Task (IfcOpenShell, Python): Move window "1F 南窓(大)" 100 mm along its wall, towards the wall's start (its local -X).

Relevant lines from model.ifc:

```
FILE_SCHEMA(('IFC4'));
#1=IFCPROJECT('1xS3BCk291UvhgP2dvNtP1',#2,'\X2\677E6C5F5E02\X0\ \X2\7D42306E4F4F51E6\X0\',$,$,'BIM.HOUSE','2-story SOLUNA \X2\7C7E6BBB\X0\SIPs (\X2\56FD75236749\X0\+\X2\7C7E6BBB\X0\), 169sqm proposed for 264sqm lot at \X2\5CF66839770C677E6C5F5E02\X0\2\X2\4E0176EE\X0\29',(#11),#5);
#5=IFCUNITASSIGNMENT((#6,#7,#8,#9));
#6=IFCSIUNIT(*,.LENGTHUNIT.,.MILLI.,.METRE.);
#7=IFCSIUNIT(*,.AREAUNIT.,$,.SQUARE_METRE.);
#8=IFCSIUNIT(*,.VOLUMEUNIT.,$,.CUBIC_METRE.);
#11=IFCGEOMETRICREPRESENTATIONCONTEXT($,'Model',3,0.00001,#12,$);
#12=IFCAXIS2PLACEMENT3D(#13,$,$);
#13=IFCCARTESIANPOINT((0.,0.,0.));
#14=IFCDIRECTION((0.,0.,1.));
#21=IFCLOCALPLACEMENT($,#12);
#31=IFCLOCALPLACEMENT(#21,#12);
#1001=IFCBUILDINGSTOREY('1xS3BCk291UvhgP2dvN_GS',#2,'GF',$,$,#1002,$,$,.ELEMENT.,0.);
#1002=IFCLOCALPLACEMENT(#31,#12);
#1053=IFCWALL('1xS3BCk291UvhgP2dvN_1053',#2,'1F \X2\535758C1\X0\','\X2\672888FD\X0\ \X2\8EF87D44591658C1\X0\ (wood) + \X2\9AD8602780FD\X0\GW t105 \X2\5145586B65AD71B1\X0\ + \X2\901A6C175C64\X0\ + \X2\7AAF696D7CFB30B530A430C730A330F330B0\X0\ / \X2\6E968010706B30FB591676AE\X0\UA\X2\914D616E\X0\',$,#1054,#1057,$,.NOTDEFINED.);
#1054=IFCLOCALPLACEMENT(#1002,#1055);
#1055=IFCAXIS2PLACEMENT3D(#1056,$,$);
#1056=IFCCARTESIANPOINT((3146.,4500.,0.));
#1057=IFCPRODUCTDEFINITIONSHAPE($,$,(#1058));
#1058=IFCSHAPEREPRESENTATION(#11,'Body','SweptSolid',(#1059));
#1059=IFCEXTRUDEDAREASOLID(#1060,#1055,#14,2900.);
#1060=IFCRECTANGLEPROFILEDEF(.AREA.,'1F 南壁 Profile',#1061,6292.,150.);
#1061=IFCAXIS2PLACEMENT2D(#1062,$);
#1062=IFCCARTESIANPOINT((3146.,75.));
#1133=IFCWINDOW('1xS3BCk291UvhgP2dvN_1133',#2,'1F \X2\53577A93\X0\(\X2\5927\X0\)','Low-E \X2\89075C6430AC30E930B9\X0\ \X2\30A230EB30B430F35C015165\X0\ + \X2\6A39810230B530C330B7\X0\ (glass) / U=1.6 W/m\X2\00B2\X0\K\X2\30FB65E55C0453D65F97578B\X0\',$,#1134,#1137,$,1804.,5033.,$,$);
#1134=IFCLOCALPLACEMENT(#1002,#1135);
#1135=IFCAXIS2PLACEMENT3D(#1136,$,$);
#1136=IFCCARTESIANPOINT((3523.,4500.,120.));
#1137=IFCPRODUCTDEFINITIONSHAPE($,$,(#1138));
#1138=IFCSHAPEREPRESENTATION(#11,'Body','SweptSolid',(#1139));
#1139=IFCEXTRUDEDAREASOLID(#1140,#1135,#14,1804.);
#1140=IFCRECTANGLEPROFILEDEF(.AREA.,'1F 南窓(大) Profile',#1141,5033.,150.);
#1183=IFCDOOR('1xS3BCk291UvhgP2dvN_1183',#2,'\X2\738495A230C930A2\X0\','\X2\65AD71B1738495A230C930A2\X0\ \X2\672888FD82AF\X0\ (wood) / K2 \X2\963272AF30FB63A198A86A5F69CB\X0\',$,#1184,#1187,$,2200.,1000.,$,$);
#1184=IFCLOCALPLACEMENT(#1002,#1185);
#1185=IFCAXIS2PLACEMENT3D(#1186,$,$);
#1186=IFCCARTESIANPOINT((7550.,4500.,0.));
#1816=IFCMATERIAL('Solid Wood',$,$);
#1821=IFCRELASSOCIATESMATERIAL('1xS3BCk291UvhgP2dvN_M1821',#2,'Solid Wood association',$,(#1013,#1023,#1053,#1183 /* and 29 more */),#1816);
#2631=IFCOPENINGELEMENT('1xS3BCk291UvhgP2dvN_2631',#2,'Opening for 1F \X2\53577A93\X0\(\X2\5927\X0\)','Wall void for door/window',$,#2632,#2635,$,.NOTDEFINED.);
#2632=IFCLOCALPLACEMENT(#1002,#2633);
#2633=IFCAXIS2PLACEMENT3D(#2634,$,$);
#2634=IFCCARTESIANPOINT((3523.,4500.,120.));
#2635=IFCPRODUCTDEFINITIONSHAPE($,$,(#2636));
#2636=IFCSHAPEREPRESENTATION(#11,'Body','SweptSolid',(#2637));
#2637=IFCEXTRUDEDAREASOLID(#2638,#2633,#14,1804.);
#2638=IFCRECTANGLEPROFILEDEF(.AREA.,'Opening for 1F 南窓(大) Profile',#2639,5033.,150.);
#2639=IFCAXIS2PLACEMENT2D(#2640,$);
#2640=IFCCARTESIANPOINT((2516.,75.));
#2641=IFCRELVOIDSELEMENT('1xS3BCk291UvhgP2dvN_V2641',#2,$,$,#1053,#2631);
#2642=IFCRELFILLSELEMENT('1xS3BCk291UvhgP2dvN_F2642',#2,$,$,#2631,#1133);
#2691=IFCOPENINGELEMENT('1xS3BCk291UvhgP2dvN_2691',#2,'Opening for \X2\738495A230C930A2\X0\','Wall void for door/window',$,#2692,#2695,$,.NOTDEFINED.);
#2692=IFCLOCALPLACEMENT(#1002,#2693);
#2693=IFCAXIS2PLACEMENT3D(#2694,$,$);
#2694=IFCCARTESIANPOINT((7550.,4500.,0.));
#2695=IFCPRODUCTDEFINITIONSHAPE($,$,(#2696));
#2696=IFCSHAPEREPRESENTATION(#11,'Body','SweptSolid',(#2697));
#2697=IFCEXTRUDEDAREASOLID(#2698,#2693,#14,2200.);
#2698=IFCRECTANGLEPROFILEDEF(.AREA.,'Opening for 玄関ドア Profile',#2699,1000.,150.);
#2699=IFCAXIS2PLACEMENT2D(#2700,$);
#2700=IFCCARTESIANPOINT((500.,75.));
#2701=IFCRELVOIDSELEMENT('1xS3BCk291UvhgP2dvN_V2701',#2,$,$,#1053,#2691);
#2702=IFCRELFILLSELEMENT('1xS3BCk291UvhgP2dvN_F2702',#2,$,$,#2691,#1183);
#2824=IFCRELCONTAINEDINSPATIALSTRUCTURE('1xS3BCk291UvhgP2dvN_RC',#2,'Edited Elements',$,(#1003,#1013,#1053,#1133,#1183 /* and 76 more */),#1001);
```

```python
import ifcopenshell
import ifcopenshell.api.geometry
import ifcopenshell.util.placement
import ifcopenshell.util.unit

model = ifcopenshell.open("model.ifc")
unit_scale = ifcopenshell.util.unit.calculate_unit_scale(model)

window = model.by_id(1133)
opening = window.FillsVoids[0].RelatingOpeningElement
wall = opening.VoidsElements[0].RelatingBuildingElement

wall_matrix = ifcopenshell.util.placement.get_local_placement(wall.ObjectPlacement)
shift = wall_matrix[:3, 0] * -0.1 / unit_scale
before = ifcopenshell.util.placement.get_local_placement(window.ObjectPlacement)[:3, 3].copy()

# The window is not placed relative to its opening, so move both.
for product in (opening, window):
    matrix = ifcopenshell.util.placement.get_local_placement(product.ObjectPlacement)
    matrix[:3, 3] += shift
    ifcopenshell.api.geometry.edit_object_placement(model, product=product, matrix=matrix, is_si=False)

after = ifcopenshell.util.placement.get_local_placement(window.ObjectPlacement)[:3, 3]
print("window moved by", (after - before).round(3) + 0.0)

model.write("model_rev.ifc")
```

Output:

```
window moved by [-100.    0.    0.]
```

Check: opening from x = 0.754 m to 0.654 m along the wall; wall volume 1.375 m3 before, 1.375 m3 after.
